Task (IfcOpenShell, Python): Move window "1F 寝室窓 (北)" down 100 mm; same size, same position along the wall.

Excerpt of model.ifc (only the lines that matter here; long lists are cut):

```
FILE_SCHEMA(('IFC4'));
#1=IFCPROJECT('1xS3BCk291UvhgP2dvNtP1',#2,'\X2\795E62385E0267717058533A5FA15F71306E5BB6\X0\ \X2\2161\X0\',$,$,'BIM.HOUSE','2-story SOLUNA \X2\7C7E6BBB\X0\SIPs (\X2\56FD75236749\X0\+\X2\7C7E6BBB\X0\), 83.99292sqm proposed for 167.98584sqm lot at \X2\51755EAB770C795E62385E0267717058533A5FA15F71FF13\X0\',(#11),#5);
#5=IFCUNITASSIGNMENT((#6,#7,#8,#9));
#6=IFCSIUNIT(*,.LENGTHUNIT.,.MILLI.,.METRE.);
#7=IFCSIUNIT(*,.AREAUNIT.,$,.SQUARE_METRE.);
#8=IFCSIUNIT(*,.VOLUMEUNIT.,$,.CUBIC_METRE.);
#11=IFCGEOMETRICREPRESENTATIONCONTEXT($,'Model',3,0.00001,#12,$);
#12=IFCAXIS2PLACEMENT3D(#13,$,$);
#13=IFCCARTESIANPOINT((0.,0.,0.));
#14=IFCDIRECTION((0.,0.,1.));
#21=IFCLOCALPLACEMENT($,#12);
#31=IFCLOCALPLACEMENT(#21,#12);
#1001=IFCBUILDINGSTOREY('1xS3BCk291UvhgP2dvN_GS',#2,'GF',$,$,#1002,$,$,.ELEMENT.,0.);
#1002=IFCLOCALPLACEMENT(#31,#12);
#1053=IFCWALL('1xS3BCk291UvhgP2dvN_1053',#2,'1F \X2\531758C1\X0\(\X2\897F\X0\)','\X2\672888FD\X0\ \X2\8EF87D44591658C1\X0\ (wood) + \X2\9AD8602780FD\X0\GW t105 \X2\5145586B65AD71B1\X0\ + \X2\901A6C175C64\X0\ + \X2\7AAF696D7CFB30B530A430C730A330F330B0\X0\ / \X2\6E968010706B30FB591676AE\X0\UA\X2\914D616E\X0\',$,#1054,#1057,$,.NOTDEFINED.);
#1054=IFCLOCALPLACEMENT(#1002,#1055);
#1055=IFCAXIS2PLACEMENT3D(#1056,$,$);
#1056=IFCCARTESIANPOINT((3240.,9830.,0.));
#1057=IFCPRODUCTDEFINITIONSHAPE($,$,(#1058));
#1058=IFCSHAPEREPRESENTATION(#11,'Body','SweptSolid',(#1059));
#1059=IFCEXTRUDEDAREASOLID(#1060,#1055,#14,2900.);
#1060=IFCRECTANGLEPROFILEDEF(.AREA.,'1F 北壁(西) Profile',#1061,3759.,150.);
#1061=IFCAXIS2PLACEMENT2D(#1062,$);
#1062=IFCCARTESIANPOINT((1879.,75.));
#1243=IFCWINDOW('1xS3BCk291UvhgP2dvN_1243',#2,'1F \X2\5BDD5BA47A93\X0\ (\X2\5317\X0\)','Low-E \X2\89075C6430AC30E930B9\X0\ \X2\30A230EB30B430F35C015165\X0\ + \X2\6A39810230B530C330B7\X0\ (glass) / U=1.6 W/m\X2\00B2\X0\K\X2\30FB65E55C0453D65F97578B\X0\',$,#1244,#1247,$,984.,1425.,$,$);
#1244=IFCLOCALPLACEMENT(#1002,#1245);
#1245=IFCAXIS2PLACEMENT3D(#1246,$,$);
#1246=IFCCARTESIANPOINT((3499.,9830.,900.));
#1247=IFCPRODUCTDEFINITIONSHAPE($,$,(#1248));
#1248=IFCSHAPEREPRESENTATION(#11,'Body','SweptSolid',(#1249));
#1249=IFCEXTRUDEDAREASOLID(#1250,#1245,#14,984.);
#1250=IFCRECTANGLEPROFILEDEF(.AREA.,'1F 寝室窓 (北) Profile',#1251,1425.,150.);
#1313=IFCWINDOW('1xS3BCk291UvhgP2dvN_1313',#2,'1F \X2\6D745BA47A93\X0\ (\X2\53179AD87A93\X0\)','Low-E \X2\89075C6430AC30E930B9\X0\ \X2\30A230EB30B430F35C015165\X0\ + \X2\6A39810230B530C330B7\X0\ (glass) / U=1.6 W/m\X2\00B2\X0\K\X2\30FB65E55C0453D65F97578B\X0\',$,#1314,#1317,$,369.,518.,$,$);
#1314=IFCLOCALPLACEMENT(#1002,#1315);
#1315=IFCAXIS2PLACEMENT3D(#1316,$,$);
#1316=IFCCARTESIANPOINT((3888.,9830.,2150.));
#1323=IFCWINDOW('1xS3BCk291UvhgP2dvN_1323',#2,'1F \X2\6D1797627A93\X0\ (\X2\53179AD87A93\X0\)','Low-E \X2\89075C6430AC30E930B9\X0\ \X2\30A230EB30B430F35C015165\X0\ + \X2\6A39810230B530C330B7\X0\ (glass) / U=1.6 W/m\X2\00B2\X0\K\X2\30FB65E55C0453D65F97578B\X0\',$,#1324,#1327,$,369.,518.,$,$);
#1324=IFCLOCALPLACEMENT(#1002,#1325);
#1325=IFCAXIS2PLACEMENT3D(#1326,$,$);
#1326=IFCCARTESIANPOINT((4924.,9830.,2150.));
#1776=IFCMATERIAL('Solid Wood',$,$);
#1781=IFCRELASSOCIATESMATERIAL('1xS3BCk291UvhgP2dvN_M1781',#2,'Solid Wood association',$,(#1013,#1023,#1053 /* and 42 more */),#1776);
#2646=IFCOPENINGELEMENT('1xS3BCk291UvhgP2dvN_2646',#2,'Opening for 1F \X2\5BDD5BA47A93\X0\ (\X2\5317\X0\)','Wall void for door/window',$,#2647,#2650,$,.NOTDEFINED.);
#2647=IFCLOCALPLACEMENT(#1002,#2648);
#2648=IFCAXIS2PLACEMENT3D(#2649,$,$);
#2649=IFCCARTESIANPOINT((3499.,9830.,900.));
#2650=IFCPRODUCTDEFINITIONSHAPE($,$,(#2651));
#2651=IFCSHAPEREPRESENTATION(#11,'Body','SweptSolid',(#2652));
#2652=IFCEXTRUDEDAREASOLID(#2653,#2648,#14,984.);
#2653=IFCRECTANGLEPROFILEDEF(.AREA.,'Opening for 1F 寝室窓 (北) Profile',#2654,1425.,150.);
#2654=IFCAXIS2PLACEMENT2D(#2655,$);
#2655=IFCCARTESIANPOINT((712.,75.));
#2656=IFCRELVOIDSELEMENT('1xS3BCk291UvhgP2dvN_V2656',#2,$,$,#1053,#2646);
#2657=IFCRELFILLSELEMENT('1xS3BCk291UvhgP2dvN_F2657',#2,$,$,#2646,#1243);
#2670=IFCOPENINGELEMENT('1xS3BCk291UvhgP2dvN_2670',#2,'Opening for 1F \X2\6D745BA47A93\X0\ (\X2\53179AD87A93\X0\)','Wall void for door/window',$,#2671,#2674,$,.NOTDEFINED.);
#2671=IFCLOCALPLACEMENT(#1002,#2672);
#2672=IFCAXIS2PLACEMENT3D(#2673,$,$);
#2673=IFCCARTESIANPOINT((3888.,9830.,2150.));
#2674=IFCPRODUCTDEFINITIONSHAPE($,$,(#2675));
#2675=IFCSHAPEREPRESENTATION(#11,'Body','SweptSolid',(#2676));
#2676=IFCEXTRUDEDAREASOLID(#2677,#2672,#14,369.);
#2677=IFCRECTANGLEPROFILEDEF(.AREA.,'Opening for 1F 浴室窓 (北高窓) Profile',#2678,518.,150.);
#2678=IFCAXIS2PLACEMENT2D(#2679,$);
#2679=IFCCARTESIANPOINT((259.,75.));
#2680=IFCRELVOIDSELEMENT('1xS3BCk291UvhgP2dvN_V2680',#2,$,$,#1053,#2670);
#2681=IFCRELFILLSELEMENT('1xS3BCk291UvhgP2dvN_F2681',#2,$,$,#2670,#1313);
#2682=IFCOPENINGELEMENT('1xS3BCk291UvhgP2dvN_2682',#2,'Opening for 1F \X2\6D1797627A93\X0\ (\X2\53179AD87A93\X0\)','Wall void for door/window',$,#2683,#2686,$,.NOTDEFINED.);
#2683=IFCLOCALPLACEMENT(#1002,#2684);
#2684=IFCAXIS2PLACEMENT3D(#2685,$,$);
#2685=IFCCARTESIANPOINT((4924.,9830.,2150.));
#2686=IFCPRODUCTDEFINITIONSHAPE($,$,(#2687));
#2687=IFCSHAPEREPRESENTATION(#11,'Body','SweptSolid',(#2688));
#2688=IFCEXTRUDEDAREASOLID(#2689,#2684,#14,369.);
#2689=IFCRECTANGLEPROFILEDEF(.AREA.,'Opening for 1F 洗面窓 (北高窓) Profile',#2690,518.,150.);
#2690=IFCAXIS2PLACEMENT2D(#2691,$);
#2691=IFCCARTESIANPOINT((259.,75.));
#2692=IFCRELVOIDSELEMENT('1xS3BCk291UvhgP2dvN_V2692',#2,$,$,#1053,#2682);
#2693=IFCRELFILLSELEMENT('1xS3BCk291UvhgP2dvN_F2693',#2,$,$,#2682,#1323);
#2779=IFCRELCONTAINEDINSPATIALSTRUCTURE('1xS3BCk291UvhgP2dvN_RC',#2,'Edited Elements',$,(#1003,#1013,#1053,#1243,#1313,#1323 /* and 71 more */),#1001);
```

```python
import numpy as np
import ifcopenshell
import ifcopenshell.api.geometry
import ifcopenshell.util.placement
import ifcopenshell.util.unit

model = ifcopenshell.open("model.ifc")
unit_scale = ifcopenshell.util.unit.calculate_unit_scale(model)

window = model.by_guid("1xS3BCk291UvhgP2dvN_1243")
opening = window.FillsVoids[0].RelatingOpeningElement
dz = -0.1 / unit_scale

shift = np.array([0.0, 0.0, dz])
# The window is not placed relative to its opening, so move both.
for product in (opening, window):
    matrix = ifcopenshell.util.placement.get_local_placement(product.ObjectPlacement)
    matrix[:3, 3] += shift
    ifcopenshell.api.geometry.edit_object_placement(model, product=product, matrix=matrix, is_si=False)

print(f"moved by {dz * unit_scale:+.3f} m")

model.write("model_updated.ifc")
```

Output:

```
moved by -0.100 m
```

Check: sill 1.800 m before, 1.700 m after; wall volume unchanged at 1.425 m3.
